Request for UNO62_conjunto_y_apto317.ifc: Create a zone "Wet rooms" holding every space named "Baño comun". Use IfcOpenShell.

First a look at what the model holds.

```python
import ifcopenshell

model = ifcopenshell.open("UNO62_conjunto_y_apto317.ifc")
print(model.schema)
seen = {}
for space in model.by_type("IfcSpace"):
    seen[space.LongName] = seen.get(space.LongName, 0) + 1
for name, count in sorted(seen.items(), key=str):
    print(count, "x", name)
print("zones:", [z.Name for z in model.by_type("IfcZone")][:20])
```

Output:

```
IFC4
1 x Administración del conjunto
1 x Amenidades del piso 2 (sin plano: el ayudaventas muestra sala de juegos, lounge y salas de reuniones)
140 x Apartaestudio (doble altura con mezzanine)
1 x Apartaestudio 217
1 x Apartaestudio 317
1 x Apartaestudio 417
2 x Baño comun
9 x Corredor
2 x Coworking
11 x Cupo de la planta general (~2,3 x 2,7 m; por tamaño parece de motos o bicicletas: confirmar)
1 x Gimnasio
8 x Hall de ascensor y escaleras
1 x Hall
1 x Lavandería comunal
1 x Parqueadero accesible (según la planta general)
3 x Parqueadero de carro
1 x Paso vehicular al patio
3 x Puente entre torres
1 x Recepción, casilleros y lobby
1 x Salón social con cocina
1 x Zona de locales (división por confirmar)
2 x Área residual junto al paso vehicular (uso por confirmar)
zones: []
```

```python
import ifcopenshell
import ifcopenshell.api.group
import ifcopenshell.api.root

model = ifcopenshell.open("UNO62_conjunto_y_apto317.ifc")

names = {"Baño comun"}
spaces = [s for s in model.by_type("IfcSpace") if s.LongName in names]

zone = ifcopenshell.api.root.create_entity(model, ifc_class="IfcZone", name="Wet rooms")
ifcopenshell.api.group.assign_group(model, products=spaces, group=zone)
print(len(spaces), "spaces in", zone.Name)

model.write("UNO62_conjunto_y_apto317_updated.ifc")
```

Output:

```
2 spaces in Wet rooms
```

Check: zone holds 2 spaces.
